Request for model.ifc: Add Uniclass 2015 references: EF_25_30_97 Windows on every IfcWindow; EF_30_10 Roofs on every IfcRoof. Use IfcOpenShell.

First a look at what the model holds.

```python
import ifcopenshell

model = ifcopenshell.open("model.ifc")
print(model.schema)
print("classifications:", [c.Name for c in model.by_type("IfcClassification")])
for ifc_class in ("IfcDoor", "IfcRoof", "IfcStair", "IfcWall", "IfcWindow"):
    print(ifc_class, len(model.by_type(ifc_class)))
```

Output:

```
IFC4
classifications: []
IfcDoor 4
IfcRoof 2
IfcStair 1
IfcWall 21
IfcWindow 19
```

```python
import ifcopenshell
import ifcopenshell.api.classification

model = ifcopenshell.open("model.ifc")

system = ifcopenshell.api.classification.add_classification(model, classification="Uniclass 2015")

codes = {
    "IfcWindow": ("EF_25_30_97", "Windows"),
    "IfcRoof": ("EF_30_10", "Roofs"),
}
for ifc_class, (code, name) in codes.items():
    products = model.by_type(ifc_class)
    ifcopenshell.api.classification.add_reference(
        model, products=products, classification=system, identification=code, name=name
    )
    print(code, len(products))

model.write("model_updated.ifc")
```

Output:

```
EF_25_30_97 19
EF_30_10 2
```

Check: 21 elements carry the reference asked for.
